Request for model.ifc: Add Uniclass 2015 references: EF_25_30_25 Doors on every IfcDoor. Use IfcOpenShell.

First a look at what the model holds.

```python
import ifcopenshell

model = ifcopenshell.open("model.ifc")
print(model.schema)
print("classifications:", [c.Name for c in model.by_type("IfcClassification")])
for ifc_class in ("IfcDoor", "IfcRoof", "IfcStair", "IfcWall", "IfcWindow"):
    print(ifc_class, len(model.by_type(ifc_class)))
```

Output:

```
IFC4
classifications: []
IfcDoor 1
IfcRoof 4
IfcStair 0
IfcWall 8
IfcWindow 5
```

```python
import ifcopenshell
import ifcopenshell.api.classification

model = ifcopenshell.open("model.ifc")

system = ifcopenshell.api.classification.add_classification(model, classification="Uniclass 2015")

codes = {
    "IfcDoor": ("EF_25_30_25", "Doors"),
}
for ifc_class, (code, name) in codes.items():
    products = model.by_type(ifc_class)
    ifcopenshell.api.classification.add_reference(
        model, products=products, classification=system, identification=code, name=name
    )
    print(code, len(products))

model.write("model_v2.ifc")
```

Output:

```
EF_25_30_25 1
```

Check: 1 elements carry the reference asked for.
